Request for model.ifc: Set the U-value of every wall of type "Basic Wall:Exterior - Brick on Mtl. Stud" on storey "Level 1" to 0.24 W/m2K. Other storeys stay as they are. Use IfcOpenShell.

First a look at what the model holds.

```python
import ifcopenshell
import ifcopenshell.util.element

model = ifcopenshell.open("model.ifc")
print(model.schema)
storey = next(s for s in model.by_type("IfcBuildingStorey") if s.Name == "Level 1")
walls = [e for e in ifcopenshell.util.element.get_decomposition(storey) if e.is_a("IfcWall")]
seen = {}
for e in walls:
    element_type = ifcopenshell.util.element.get_type(e)
    key = (element_type.Name if element_type != e and element_type else None, ifcopenshell.util.element.get_pset(e, "Pset_WallCommon", "ThermalTransmittance"))
    seen[key] = seen.get(key, 0) + 1
for (name, value), count in sorted(seen.items(), key=str):
    print(count, "x", name, "|", value)
```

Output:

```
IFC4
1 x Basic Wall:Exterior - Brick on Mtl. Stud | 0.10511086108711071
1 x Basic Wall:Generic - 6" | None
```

```python
import ifcopenshell
import ifcopenshell.api.pset
import ifcopenshell.util.element

model = ifcopenshell.open("model.ifc")

storey = next(s for s in model.by_type("IfcBuildingStorey") if s.Name == "Level 1")
walls = [e for e in ifcopenshell.util.element.get_decomposition(storey) if e.is_a("IfcWall")]

count = 0
for e in walls:
    element_type = ifcopenshell.util.element.get_type(e)
    if element_type in (None, e) or element_type.Name != "Basic Wall:Exterior - Brick on Mtl. Stud":
        continue
    # add_pset returns the element's existing set when there is one.
    pset = ifcopenshell.api.pset.add_pset(model, product=e, name="Pset_WallCommon")
    ifcopenshell.api.pset.edit_pset(model, pset=pset, properties={"ThermalTransmittance": 0.24})
    count += 1

print(count, "walls updated")

model.write("model-out.ifc")
```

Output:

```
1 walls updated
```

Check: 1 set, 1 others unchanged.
